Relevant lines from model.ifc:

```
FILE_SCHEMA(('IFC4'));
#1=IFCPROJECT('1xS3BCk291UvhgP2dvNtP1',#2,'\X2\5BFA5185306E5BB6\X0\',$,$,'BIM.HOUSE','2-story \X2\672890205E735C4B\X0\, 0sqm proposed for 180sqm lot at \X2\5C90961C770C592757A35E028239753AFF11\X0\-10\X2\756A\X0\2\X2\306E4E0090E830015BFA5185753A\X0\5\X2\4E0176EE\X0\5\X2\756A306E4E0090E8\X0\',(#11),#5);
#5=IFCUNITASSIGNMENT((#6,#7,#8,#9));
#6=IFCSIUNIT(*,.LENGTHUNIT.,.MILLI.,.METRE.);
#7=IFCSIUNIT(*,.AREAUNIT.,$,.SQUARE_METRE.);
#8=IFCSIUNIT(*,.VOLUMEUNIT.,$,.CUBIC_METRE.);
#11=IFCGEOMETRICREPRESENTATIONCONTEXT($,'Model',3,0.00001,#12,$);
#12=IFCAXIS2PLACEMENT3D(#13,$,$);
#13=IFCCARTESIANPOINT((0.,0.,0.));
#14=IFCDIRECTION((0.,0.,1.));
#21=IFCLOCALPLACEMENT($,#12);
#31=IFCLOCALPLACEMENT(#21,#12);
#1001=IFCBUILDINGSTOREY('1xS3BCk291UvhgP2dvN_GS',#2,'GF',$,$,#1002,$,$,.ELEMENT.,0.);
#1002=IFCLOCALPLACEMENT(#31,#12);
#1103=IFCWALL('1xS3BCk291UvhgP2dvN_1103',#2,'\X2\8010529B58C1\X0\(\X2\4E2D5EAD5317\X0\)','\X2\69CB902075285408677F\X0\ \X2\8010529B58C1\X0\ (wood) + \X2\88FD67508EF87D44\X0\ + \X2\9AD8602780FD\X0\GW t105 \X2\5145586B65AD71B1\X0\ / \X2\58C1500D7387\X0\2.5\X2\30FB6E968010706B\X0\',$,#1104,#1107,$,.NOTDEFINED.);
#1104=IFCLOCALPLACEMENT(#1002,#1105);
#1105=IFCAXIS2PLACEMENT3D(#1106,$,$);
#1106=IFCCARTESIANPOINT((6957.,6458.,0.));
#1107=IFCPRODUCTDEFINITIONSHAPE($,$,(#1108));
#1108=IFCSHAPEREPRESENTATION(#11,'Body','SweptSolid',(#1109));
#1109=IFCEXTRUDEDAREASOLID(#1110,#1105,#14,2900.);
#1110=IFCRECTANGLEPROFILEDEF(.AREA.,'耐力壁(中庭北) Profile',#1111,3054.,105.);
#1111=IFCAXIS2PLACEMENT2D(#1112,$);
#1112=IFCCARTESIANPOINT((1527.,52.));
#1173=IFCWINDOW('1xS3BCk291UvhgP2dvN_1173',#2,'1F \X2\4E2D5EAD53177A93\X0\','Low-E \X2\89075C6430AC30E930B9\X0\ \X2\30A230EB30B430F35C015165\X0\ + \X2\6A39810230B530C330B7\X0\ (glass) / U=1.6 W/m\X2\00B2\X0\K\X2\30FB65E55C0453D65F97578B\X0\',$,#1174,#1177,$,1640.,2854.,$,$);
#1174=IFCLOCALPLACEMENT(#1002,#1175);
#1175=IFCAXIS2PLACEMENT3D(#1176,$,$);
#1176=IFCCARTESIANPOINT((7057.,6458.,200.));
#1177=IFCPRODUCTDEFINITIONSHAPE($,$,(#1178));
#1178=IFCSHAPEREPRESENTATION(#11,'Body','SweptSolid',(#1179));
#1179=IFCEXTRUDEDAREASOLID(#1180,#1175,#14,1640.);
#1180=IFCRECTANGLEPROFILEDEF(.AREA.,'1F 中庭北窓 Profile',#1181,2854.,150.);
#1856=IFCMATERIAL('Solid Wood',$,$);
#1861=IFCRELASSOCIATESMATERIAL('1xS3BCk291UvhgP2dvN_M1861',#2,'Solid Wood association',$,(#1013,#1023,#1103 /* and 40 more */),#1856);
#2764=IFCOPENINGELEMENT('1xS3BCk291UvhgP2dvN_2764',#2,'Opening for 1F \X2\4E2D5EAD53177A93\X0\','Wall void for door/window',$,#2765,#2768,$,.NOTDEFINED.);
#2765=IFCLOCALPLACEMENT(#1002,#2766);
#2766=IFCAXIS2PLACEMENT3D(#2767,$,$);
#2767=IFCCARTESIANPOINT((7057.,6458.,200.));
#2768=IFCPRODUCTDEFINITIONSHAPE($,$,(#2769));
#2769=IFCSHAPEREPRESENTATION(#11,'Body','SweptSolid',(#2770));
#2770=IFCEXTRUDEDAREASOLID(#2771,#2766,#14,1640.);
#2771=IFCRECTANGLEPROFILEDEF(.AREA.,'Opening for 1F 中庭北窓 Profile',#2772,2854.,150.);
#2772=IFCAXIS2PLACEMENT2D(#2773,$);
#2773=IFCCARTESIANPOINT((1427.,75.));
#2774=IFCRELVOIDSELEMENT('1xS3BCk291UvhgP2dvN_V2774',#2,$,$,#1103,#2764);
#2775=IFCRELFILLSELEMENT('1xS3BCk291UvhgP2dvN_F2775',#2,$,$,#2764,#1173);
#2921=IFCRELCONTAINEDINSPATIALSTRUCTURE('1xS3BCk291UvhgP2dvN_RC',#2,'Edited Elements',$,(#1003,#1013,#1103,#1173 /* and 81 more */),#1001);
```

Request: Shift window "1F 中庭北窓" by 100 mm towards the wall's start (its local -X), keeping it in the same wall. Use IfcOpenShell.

```python
import ifcopenshell
import ifcopenshell.api.geometry
import ifcopenshell.util.placement
import ifcopenshell.util.unit

model = ifcopenshell.open("model.ifc")
unit_scale = ifcopenshell.util.unit.calculate_unit_scale(model)

window = model.by_guid("1xS3BCk291UvhgP2dvN_1173")
opening = window.FillsVoids[0].RelatingOpeningElement
wall = opening.VoidsElements[0].RelatingBuildingElement

wall_matrix = ifcopenshell.util.placement.get_local_placement(wall.ObjectPlacement)
shift = wall_matrix[:3, 0] * -0.1 / unit_scale
before = ifcopenshell.util.placement.get_local_placement(window.ObjectPlacement)[:3, 3].copy()

# The window is not placed relative to its opening, so move both.
for product in (opening, window):
    matrix = ifcopenshell.util.placement.get_local_placement(product.ObjectPlacement)
    matrix[:3, 3] += shift
    ifcopenshell.api.geometry.edit_object_placement(model, product=product, matrix=matrix, is_si=False)

after = ifcopenshell.util.placement.get_local_placement(window.ObjectPlacement)[:3, 3]
print("window moved by", (after - before).round(3) + 0.0)

model.write("model_rev.ifc")
```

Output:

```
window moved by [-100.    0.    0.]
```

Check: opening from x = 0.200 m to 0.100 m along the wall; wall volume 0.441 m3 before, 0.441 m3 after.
